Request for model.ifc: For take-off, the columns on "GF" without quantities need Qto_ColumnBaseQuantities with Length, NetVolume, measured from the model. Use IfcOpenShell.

First a look at what the model holds.

```python
import ifcopenshell
import ifcopenshell.util.element
import ifcopenshell.util.unit

model = ifcopenshell.open("model.ifc")
print(model.schema)
for unit_type in ("LENGTHUNIT", "AREAUNIT", "VOLUMEUNIT"):
    print(unit_type, ifcopenshell.util.unit.calculate_unit_scale(model, unit_type))
storey = next(s for s in model.by_type("IfcBuildingStorey") if s.Name == "GF")
columns = [e for e in ifcopenshell.util.element.get_decomposition(storey) if e.is_a("IfcColumn")]
for e in sorted(columns, key=lambda e: e.id()):
    print(e.id(), e.is_a(), e.Name, list(ifcopenshell.util.element.get_psets(e, qtos_only=True)), sep=" | ")
```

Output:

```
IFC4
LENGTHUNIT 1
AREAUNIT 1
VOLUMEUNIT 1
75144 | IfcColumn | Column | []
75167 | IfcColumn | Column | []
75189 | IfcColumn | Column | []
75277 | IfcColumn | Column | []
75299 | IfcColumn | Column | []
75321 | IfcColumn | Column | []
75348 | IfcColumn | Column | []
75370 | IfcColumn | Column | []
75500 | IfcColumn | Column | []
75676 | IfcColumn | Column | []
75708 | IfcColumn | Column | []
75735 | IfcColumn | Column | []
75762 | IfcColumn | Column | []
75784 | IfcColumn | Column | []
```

```python
import ifcopenshell
import ifcopenshell.api.pset
import ifcopenshell.geom
import ifcopenshell.util.element
import ifcopenshell.util.shape
import ifcopenshell.util.unit

model = ifcopenshell.open("model.ifc")
unit_scale = ifcopenshell.util.unit.calculate_unit_scale(model)
volume_scale = ifcopenshell.util.unit.calculate_unit_scale(model, "VOLUMEUNIT")
settings = ifcopenshell.geom.settings()

storey = next(s for s in model.by_type("IfcBuildingStorey") if s.Name == "GF")
columns = [e for e in ifcopenshell.util.element.get_decomposition(storey) if e.is_a("IfcColumn")]

for e in sorted(columns, key=lambda e: e.id()):
    if ifcopenshell.util.element.get_psets(e, qtos_only=True, should_inherit=False):
        continue
    # Geometry comes back in metres, in the element's own axes.
    shape = ifcopenshell.geom.create_shape(settings, e)
    values = {
        "Length": ifcopenshell.util.shape.get_z(shape.geometry) / unit_scale,
        "NetVolume": ifcopenshell.util.shape.get_volume(shape.geometry) / volume_scale,
    }
    qto = ifcopenshell.api.pset.add_qto(model, product=e, name="Qto_ColumnBaseQuantities")
    ifcopenshell.api.pset.edit_qto(model, qto=qto, properties=values)
    print(e.id(), {k: round(v, 3) for k, v in values.items()})

model.write("model_edited.ifc")
```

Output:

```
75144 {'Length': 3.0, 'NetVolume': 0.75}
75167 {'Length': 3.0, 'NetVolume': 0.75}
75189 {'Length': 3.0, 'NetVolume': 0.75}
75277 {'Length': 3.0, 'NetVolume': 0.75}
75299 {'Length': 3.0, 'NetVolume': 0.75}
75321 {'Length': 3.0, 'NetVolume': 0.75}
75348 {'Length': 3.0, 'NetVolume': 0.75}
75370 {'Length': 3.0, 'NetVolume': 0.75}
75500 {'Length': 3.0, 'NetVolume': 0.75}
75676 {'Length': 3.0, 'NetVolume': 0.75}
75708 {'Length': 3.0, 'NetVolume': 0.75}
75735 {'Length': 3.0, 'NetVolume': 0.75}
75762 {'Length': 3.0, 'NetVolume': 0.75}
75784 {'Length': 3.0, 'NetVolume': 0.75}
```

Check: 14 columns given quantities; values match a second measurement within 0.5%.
